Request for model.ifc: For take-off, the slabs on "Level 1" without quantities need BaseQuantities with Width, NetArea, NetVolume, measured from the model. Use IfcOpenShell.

First a look at what the model holds.

```python
import ifcopenshell
import ifcopenshell.util.element
import ifcopenshell.util.unit

model = ifcopenshell.open("model.ifc")
print(model.schema)
for unit_type in ("LENGTHUNIT", "AREAUNIT", "VOLUMEUNIT"):
    print(unit_type, ifcopenshell.util.unit.calculate_unit_scale(model, unit_type))
storey = next(s for s in model.by_type("IfcBuildingStorey") if s.Name == "Level 1")
slabs = [e for e in ifcopenshell.util.element.get_decomposition(storey) if e.is_a("IfcSlab")]
for e in sorted(slabs, key=lambda e: e.id()):
    print(e.id(), e.is_a(), e.Name, list(ifcopenshell.util.element.get_psets(e, qtos_only=True)), sep=" | ")
```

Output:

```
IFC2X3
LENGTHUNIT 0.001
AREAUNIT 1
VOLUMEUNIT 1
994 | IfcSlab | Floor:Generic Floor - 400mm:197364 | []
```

```python
import ifcopenshell
import ifcopenshell.api.pset
import ifcopenshell.geom
import ifcopenshell.util.element
import ifcopenshell.util.shape
import ifcopenshell.util.unit

model = ifcopenshell.open("model.ifc")
unit_scale = ifcopenshell.util.unit.calculate_unit_scale(model)
area_scale = ifcopenshell.util.unit.calculate_unit_scale(model, "AREAUNIT")
volume_scale = ifcopenshell.util.unit.calculate_unit_scale(model, "VOLUMEUNIT")
settings = ifcopenshell.geom.settings()

storey = next(s for s in model.by_type("IfcBuildingStorey") if s.Name == "Level 1")
slabs = [e for e in ifcopenshell.util.element.get_decomposition(storey) if e.is_a("IfcSlab")]

for e in sorted(slabs, key=lambda e: e.id()):
    if ifcopenshell.util.element.get_psets(e, qtos_only=True, should_inherit=False):
        continue
    # Geometry comes back in metres, in the element's own axes.
    shape = ifcopenshell.geom.create_shape(settings, e)
    values = {
        "Width": ifcopenshell.util.shape.get_z(shape.geometry) / unit_scale,
        "NetArea": ifcopenshell.util.shape.get_footprint_area(shape.geometry) / area_scale,
        "NetVolume": ifcopenshell.util.shape.get_volume(shape.geometry) / volume_scale,
    }
    qto = ifcopenshell.api.pset.add_qto(model, product=e, name="BaseQuantities")
    ifcopenshell.api.pset.edit_qto(model, qto=qto, properties=values)
    print(e.id(), {k: round(v, 3) for k, v in values.items()})

model.write("model_rev.ifc")
```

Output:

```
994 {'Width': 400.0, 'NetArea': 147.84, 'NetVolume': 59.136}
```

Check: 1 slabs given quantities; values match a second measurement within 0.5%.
